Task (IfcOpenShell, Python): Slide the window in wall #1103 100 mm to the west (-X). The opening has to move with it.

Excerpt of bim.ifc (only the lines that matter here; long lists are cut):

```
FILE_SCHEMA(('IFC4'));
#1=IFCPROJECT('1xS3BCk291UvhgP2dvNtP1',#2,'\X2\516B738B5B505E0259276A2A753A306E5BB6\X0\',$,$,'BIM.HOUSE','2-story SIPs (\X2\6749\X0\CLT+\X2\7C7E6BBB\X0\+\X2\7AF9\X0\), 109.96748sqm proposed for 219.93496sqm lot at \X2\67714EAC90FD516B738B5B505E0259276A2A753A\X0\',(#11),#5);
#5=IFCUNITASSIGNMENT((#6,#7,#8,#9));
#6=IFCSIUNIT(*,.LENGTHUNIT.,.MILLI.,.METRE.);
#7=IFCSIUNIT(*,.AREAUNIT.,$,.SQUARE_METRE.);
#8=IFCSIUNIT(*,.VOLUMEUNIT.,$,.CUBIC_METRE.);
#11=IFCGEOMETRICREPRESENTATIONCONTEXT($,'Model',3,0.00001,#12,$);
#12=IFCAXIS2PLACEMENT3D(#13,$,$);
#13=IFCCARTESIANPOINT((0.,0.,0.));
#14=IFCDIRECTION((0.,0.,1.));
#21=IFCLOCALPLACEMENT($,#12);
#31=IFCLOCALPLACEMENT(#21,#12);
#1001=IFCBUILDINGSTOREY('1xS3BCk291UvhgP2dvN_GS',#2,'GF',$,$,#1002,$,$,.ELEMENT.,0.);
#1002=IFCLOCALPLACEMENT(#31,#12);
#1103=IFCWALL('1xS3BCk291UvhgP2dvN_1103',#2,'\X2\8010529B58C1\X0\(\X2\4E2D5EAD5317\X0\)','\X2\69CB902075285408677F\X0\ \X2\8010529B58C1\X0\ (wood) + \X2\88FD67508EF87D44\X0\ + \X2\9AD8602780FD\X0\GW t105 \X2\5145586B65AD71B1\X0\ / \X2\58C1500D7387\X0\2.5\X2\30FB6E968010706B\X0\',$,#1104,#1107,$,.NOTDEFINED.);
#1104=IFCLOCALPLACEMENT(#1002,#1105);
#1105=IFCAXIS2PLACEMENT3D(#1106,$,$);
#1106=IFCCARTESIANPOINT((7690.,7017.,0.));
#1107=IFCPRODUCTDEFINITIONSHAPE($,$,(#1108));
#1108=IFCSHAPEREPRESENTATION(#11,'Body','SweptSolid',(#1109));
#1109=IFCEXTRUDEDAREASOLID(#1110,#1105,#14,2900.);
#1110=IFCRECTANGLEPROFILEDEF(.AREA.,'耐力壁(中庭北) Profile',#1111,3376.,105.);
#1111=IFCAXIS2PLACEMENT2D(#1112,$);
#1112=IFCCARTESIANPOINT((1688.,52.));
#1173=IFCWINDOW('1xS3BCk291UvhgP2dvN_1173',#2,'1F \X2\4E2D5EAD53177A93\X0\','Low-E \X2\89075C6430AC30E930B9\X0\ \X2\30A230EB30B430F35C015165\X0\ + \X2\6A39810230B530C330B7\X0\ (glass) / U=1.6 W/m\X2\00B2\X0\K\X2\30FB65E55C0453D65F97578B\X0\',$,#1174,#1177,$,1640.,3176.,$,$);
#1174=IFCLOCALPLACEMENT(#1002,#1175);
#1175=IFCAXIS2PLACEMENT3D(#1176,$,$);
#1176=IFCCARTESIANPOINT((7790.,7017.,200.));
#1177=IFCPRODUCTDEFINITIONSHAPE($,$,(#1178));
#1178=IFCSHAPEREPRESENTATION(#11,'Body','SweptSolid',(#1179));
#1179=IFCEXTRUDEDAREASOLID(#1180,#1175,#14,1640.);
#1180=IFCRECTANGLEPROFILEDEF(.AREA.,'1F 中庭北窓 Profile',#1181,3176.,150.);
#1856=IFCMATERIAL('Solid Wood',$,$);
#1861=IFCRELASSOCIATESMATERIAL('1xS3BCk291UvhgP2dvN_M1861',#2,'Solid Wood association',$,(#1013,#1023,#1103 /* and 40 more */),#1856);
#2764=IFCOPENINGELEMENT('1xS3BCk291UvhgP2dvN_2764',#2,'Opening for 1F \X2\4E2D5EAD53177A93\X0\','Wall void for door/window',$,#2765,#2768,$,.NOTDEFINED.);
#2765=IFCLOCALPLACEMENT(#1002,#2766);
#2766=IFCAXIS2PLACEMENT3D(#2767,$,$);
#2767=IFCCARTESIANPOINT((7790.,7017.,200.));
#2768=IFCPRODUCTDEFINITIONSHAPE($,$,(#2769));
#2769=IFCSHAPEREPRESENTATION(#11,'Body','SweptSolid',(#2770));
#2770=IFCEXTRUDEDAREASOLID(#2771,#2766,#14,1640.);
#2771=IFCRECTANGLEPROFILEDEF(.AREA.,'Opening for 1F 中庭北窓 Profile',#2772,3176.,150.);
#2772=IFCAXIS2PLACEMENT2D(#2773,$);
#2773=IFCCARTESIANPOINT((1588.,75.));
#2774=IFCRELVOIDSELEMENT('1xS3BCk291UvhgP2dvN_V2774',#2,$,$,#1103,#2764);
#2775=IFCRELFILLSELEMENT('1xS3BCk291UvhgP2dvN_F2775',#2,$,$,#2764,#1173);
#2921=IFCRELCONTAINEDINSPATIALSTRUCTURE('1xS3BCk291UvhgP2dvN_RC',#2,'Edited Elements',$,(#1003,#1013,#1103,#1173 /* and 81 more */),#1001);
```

```python
import ifcopenshell
import ifcopenshell.api.geometry
import ifcopenshell.util.placement
import ifcopenshell.util.unit

model = ifcopenshell.open("bim.ifc")
unit_scale = ifcopenshell.util.unit.calculate_unit_scale(model)

window = model.by_guid("1xS3BCk291UvhgP2dvN_1173")
opening = window.FillsVoids[0].RelatingOpeningElement
wall = opening.VoidsElements[0].RelatingBuildingElement

wall_matrix = ifcopenshell.util.placement.get_local_placement(wall.ObjectPlacement)
shift = wall_matrix[:3, 0] * -0.1 / unit_scale
before = ifcopenshell.util.placement.get_local_placement(window.ObjectPlacement)[:3, 3].copy()

# The window is not placed relative to its opening, so move both.
for product in (opening, window):
    matrix = ifcopenshell.util.placement.get_local_placement(product.ObjectPlacement)
    matrix[:3, 3] += shift
    ifcopenshell.api.geometry.edit_object_placement(model, product=product, matrix=matrix, is_si=False)

after = ifcopenshell.util.placement.get_local_placement(window.ObjectPlacement)[:3, 3]
print("window moved by", (after - before).round(3) + 0.0)

model.write("bim_updated.ifc")
```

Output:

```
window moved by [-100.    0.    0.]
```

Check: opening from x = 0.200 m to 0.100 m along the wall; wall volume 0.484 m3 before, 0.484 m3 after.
